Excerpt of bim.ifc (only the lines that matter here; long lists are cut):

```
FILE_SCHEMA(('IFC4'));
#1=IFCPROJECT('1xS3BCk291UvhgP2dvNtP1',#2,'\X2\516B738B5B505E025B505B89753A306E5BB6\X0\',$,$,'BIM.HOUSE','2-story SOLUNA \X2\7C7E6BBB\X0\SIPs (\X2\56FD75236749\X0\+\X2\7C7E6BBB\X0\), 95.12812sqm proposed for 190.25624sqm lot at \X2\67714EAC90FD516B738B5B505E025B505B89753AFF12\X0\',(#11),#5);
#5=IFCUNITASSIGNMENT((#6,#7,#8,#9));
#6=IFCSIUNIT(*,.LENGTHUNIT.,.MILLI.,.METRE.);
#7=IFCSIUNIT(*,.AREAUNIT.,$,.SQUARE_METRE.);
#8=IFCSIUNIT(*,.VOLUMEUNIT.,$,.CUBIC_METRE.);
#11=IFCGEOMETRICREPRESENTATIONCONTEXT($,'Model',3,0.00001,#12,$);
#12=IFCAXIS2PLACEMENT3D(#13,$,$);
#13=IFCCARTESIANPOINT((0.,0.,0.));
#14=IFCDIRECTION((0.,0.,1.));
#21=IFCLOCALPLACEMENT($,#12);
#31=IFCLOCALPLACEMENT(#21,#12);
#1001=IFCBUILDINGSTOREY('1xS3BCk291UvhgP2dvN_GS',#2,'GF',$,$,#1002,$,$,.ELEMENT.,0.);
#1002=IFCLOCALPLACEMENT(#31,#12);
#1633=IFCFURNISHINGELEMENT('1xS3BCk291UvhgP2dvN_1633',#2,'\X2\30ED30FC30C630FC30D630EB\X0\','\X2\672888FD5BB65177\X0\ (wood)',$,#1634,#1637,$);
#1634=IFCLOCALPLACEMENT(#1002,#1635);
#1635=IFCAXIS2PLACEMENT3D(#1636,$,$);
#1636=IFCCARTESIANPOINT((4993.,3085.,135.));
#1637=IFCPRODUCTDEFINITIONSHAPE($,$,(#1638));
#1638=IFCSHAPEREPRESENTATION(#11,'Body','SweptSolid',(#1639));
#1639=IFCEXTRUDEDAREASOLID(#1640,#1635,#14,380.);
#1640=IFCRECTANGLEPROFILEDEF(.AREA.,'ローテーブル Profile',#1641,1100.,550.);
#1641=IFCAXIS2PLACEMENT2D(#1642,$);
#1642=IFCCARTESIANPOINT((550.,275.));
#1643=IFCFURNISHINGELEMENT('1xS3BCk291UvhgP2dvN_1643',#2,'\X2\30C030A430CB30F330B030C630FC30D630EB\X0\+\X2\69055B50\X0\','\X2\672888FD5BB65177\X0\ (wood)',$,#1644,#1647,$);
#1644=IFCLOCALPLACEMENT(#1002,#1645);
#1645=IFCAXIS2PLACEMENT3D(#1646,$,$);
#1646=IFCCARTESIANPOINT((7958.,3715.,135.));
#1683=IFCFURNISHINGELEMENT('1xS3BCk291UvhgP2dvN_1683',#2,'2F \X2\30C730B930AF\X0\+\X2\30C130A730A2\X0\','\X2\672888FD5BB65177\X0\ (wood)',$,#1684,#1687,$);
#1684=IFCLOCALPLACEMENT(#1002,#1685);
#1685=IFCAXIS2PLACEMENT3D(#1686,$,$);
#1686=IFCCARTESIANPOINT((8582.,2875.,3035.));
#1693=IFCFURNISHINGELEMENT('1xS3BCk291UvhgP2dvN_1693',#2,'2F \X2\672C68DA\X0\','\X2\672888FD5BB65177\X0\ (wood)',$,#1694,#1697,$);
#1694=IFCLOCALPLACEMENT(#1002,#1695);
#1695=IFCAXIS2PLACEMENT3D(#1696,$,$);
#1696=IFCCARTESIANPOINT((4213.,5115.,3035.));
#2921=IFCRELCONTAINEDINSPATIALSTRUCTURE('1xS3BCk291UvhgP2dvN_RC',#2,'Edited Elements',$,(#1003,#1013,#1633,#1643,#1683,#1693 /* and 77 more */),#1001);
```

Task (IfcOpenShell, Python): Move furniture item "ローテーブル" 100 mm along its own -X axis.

```python
import ifcopenshell
import ifcopenshell.api.geometry
import ifcopenshell.util.placement
import ifcopenshell.util.unit

model = ifcopenshell.open("bim.ifc")
unit_scale = ifcopenshell.util.unit.calculate_unit_scale(model)

item = model.by_guid("1xS3BCk291UvhgP2dvN_1633")
matrix = ifcopenshell.util.placement.get_local_placement(item.ObjectPlacement)
matrix[:3, 3] -= matrix[:3, 0] * 0.1 / unit_scale
ifcopenshell.api.geometry.edit_object_placement(model, product=item, matrix=matrix, is_si=False)

print(ifcopenshell.util.placement.get_local_placement(item.ObjectPlacement).round(3) + 0.0)

model.write("bim-out.ifc")
```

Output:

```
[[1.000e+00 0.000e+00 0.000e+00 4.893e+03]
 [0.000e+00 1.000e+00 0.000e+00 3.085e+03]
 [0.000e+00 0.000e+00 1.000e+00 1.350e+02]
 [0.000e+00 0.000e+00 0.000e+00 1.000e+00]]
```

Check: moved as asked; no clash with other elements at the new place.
